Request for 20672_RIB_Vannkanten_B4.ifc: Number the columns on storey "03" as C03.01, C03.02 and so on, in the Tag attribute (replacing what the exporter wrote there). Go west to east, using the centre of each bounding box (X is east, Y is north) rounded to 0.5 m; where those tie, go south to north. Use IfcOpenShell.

First a look at what the model holds.

```python
import ifcopenshell
import ifcopenshell.util.element
import ifcopenshell.util.placement

model = ifcopenshell.open("20672_RIB_Vannkanten_B4.ifc")
print(model.schema)
storey = next(s for s in model.by_type("IfcBuildingStorey") if s.Name == "03")
columns = [e for e in ifcopenshell.util.element.get_decomposition(storey) if e.is_a("IfcColumn")]
for e in sorted(columns, key=lambda e: e.id()):
    origin = ifcopenshell.util.placement.get_local_placement(e.ObjectPlacement)[:3, 3]
    print(e.id(), e.Tag, e.Name, origin.round(2) + 0.0, sep=" | ")
```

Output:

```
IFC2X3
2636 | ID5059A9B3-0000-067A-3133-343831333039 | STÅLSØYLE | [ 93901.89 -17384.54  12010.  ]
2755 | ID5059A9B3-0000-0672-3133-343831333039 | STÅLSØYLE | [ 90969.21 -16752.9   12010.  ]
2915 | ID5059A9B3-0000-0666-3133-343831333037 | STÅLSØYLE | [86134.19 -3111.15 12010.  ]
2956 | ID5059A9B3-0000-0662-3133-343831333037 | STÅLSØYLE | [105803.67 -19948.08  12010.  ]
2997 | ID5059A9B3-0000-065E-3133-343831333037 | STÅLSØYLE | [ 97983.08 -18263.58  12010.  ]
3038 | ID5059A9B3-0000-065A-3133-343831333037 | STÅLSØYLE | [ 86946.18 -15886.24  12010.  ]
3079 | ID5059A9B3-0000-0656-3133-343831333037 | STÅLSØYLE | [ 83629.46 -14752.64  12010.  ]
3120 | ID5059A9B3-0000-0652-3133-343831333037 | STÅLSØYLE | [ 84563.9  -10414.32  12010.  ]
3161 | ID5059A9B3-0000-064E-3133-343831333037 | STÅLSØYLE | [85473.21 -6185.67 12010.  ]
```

```python
import ifcopenshell
import ifcopenshell.geom
import ifcopenshell.util.element
import ifcopenshell.util.shape

model = ifcopenshell.open("20672_RIB_Vannkanten_B4.ifc")
settings = ifcopenshell.geom.settings()
settings.set("use-world-coords", True)


def centre(element):
    shape = ifcopenshell.geom.create_shape(settings, element)
    return ifcopenshell.util.shape.get_bbox_centroid(shape.geometry)


storey = next(s for s in model.by_type("IfcBuildingStorey") if s.Name == "03")
columns = [e for e in ifcopenshell.util.element.get_decomposition(storey) if e.is_a("IfcColumn")]

# Insertion points can sit at a corner or the storey origin, so sort by the geometry (in metres).
centres = {e: centre(e) for e in columns}
columns.sort(key=lambda e: (round(centres[e][0] / 0.5), centres[e][1]))

for i, e in enumerate(columns, start=1):
    number = f"C03.{i:02d}"
    e.Tag = number
    print(e.id(), number)

model.write("20672_RIB_Vannkanten_B4_updated.ifc")
```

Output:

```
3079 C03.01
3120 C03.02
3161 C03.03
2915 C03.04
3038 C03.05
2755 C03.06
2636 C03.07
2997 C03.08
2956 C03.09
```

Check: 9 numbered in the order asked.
